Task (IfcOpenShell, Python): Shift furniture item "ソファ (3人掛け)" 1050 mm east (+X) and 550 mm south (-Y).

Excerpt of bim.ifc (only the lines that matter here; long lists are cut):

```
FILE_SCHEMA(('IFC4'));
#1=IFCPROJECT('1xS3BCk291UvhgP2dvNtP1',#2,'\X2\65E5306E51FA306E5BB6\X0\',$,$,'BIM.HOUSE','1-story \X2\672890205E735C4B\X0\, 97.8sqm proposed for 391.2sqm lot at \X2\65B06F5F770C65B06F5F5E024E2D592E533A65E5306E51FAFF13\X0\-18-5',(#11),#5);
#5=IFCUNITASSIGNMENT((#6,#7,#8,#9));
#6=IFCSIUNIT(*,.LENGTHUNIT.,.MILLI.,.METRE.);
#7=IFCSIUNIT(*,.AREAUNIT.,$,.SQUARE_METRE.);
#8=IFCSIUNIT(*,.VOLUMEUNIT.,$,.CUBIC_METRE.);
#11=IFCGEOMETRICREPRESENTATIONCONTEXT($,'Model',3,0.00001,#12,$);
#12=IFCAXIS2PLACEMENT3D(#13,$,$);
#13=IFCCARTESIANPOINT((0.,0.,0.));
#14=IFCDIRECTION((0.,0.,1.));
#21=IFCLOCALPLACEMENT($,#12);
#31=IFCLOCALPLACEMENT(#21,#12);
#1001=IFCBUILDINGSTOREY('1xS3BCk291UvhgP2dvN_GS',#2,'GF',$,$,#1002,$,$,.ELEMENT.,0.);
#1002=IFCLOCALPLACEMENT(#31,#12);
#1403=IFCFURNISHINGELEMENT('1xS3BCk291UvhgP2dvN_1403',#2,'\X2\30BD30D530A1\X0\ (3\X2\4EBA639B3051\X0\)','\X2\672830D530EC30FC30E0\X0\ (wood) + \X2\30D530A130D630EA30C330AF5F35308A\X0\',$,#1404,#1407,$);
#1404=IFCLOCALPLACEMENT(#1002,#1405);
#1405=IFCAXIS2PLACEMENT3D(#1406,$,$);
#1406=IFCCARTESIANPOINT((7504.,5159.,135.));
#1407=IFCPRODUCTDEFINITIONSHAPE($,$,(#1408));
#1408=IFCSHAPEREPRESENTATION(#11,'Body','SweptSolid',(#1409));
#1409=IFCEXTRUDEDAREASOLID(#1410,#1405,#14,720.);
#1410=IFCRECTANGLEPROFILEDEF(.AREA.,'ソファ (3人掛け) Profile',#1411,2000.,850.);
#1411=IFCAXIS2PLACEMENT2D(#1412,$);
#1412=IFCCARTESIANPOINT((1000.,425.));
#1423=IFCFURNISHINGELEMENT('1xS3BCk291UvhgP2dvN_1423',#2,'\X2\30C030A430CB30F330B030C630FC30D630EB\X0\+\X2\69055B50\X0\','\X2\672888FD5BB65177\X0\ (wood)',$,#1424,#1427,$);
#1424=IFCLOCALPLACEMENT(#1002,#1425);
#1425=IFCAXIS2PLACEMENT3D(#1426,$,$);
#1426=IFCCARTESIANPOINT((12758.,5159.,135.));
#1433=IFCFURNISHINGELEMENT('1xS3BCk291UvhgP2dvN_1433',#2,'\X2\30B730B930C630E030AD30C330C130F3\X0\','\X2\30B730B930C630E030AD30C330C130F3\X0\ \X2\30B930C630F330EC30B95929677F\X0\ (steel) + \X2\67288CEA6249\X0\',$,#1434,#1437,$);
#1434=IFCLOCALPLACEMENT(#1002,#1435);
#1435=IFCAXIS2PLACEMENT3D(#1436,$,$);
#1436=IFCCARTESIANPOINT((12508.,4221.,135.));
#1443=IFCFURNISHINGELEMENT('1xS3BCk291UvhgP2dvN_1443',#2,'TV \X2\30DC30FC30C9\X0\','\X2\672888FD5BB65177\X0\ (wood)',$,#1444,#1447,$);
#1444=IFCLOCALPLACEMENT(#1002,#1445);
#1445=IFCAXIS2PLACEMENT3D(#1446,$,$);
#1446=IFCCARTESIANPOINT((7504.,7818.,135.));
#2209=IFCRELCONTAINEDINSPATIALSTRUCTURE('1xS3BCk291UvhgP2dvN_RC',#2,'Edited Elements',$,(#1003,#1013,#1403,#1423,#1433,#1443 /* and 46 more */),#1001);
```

```python
import ifcopenshell
import ifcopenshell.api.geometry
import ifcopenshell.util.placement

model = ifcopenshell.open("bim.ifc")

item = model.by_guid("1xS3BCk291UvhgP2dvN_1403")
matrix = ifcopenshell.util.placement.get_local_placement(item.ObjectPlacement)
matrix[0, 3] += 1050.0
matrix[1, 3] -= 550.0
ifcopenshell.api.geometry.edit_object_placement(model, product=item, matrix=matrix, is_si=False)

print(ifcopenshell.util.placement.get_local_placement(item.ObjectPlacement).round(3) + 0.0)

model.write("bim_rev.ifc")
```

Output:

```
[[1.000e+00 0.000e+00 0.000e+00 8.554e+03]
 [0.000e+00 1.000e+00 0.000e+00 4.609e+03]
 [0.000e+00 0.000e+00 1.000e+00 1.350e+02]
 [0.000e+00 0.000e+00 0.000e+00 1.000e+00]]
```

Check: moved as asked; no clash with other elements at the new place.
